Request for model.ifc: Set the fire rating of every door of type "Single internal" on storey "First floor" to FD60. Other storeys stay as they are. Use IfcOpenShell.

First a look at what the model holds.

```python
import ifcopenshell
import ifcopenshell.util.element

model = ifcopenshell.open("model.ifc")
print(model.schema)
storey = next(s for s in model.by_type("IfcBuildingStorey") if s.Name == "First floor")
doors = [e for e in ifcopenshell.util.element.get_decomposition(storey) if e.is_a("IfcDoor")]
seen = {}
for e in doors:
    element_type = ifcopenshell.util.element.get_type(e)
    key = (element_type.Name if element_type != e and element_type else None, ifcopenshell.util.element.get_pset(e, "Pset_DoorCommon", "FireRating"))
    seen[key] = seen.get(key, 0) + 1
for (name, value), count in sorted(seen.items(), key=str):
    print(count, "x", name, "|", value)
```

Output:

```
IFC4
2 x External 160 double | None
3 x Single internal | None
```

```python
import ifcopenshell
import ifcopenshell.api.pset
import ifcopenshell.util.element

model = ifcopenshell.open("model.ifc")

storey = next(s for s in model.by_type("IfcBuildingStorey") if s.Name == "First floor")
doors = [e for e in ifcopenshell.util.element.get_decomposition(storey) if e.is_a("IfcDoor")]

count = 0
for e in doors:
    element_type = ifcopenshell.util.element.get_type(e)
    if element_type in (None, e) or element_type.Name != "Single internal":
        continue
    # add_pset returns the element's existing set when there is one.
    pset = ifcopenshell.api.pset.add_pset(model, product=e, name="Pset_DoorCommon")
    ifcopenshell.api.pset.edit_pset(model, pset=pset, properties={"FireRating": "FD60"})
    count += 1

print(count, "doors updated")

model.write("model-out.ifc")
```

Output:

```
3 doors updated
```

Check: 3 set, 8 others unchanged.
